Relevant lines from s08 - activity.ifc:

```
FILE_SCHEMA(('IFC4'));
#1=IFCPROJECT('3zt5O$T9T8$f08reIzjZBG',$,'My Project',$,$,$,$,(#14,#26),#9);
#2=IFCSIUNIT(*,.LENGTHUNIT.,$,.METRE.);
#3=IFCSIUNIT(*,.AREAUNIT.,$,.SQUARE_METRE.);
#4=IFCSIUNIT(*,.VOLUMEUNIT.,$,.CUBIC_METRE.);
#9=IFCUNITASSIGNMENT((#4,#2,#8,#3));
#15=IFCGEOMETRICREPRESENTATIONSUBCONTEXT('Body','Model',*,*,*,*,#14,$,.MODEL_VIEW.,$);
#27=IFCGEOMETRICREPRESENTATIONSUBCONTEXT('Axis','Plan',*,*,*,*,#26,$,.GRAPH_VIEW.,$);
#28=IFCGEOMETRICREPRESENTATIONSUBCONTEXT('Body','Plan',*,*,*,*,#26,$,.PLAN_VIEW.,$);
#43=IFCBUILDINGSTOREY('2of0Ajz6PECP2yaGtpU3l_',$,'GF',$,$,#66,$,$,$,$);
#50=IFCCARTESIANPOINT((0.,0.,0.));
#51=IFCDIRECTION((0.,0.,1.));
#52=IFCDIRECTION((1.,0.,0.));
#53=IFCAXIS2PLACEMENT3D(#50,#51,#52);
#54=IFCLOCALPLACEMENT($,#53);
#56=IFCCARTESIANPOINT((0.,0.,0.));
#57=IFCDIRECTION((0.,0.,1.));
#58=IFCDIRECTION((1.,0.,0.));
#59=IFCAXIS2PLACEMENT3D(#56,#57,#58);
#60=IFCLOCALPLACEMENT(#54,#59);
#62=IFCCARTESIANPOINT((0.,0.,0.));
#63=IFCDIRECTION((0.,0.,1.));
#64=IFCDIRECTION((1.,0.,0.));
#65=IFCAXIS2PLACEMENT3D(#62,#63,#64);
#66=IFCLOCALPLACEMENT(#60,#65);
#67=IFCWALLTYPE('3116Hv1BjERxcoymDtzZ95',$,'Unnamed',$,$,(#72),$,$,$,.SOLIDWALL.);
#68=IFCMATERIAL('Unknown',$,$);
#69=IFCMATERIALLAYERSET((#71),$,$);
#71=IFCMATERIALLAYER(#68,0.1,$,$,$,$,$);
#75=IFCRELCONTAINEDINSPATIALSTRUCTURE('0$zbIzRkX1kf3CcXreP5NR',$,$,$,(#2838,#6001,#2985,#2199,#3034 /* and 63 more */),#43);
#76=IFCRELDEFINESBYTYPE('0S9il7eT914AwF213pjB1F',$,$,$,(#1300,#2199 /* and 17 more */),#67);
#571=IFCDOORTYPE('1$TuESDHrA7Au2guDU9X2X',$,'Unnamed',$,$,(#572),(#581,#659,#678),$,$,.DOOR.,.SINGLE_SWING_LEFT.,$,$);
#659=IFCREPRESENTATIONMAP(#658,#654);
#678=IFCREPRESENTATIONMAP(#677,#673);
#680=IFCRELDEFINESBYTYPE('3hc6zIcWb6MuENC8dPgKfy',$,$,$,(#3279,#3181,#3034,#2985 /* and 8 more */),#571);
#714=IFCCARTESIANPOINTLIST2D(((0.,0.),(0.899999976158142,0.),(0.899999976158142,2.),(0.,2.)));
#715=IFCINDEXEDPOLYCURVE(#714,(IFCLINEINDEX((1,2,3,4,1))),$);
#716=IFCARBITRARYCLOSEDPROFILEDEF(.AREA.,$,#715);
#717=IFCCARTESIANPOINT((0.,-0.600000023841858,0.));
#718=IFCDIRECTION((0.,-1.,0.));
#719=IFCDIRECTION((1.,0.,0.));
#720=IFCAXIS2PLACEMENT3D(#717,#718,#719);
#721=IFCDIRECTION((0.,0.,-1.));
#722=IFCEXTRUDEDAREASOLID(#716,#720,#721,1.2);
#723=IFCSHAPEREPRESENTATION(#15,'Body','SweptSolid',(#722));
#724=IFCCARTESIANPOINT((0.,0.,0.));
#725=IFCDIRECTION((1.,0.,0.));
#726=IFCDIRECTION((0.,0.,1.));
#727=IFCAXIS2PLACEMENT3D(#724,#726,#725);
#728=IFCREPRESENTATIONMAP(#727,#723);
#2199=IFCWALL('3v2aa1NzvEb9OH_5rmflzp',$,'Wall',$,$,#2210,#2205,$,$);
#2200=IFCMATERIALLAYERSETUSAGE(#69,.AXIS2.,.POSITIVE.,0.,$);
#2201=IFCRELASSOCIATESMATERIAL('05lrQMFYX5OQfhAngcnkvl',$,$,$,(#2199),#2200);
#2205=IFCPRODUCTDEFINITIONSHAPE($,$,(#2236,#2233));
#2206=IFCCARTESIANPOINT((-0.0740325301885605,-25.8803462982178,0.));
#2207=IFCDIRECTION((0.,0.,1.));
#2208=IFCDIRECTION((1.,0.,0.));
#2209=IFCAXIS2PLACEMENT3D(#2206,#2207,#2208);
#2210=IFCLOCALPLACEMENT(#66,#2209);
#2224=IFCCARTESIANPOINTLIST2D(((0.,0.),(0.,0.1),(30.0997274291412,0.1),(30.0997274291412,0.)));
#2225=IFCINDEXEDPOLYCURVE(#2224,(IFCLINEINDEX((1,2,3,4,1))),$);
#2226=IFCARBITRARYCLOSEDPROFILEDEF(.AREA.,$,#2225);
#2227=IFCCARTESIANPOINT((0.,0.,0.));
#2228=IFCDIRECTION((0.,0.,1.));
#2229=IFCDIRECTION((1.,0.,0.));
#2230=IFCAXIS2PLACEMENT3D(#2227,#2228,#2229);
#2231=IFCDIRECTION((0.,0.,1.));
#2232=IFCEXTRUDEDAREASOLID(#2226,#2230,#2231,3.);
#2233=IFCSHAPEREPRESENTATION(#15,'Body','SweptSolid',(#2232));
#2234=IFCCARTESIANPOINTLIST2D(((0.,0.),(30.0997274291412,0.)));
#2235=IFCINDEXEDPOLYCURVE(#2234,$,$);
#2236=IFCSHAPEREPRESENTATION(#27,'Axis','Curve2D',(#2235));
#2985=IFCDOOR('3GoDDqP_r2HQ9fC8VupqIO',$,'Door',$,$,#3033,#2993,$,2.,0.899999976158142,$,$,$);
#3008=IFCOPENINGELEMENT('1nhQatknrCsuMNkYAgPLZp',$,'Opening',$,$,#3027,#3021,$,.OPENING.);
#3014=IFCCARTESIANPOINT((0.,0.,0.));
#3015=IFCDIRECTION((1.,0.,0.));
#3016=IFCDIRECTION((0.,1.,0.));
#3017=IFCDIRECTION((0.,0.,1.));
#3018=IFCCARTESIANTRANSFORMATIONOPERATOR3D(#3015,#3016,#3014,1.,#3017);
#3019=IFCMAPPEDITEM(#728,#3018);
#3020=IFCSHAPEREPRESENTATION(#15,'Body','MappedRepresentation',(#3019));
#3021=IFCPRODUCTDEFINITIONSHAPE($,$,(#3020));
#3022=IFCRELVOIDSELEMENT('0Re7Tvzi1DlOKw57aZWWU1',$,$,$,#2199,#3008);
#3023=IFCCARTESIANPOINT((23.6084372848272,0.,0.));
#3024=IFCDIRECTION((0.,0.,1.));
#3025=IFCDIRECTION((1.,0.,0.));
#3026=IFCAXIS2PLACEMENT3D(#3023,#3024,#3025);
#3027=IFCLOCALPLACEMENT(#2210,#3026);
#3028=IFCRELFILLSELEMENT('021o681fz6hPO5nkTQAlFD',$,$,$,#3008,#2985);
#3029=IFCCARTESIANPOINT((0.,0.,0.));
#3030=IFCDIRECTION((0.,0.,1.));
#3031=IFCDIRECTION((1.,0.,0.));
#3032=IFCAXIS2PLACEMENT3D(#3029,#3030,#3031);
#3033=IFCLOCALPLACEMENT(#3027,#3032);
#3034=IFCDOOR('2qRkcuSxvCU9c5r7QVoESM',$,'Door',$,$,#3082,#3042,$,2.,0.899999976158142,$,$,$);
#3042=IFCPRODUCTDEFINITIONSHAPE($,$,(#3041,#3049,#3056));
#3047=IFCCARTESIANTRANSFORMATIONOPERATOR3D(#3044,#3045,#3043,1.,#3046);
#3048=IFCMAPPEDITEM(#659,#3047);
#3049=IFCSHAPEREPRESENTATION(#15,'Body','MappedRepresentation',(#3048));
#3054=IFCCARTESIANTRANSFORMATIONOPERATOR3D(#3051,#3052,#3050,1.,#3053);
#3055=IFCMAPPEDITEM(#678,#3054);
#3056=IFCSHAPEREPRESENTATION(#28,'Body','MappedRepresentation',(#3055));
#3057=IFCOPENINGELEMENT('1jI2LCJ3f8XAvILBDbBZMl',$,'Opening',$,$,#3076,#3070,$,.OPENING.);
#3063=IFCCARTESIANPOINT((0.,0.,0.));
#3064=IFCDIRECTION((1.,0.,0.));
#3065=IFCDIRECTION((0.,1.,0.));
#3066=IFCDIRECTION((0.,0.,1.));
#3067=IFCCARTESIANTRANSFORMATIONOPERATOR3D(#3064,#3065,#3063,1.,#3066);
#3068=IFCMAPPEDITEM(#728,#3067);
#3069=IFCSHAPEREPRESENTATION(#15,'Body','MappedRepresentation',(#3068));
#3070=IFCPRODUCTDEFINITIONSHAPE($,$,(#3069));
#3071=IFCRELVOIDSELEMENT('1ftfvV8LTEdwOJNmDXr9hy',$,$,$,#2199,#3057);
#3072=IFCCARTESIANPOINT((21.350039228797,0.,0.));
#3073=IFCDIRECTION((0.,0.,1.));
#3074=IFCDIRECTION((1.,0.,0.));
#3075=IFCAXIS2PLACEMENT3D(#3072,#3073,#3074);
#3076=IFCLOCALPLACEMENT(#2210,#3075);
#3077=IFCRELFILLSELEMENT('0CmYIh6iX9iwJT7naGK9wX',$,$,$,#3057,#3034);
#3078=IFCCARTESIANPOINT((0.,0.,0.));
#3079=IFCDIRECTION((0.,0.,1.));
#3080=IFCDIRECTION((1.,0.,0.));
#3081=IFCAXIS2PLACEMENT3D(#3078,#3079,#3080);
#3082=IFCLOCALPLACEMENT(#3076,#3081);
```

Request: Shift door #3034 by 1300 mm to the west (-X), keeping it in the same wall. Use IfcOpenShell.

```python
import ifcopenshell
import ifcopenshell.api.geometry
import ifcopenshell.util.placement

model = ifcopenshell.open("s08 - activity.ifc")

door = model.by_guid("2qRkcuSxvCU9c5r7QVoESM")
opening = door.FillsVoids[0].RelatingOpeningElement
wall = opening.VoidsElements[0].RelatingBuildingElement

wall_matrix = ifcopenshell.util.placement.get_local_placement(wall.ObjectPlacement)
shift = wall_matrix[:3, 0] * -1.3
before = ifcopenshell.util.placement.get_local_placement(door.ObjectPlacement)[:3, 3].copy()

# The door is placed relative to its opening, so it follows when the opening moves.
matrix = ifcopenshell.util.placement.get_local_placement(opening.ObjectPlacement)
matrix[:3, 3] += shift
ifcopenshell.api.geometry.edit_object_placement(
    model, product=opening, matrix=matrix, is_si=False, should_transform_children=True
)

after = ifcopenshell.util.placement.get_local_placement(door.ObjectPlacement)[:3, 3]
print("door moved by", (after - before).round(3) + 0.0)

model.write("s08 - activity_v2.ifc")
```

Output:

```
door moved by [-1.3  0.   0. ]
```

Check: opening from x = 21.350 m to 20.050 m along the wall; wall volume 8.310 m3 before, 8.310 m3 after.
